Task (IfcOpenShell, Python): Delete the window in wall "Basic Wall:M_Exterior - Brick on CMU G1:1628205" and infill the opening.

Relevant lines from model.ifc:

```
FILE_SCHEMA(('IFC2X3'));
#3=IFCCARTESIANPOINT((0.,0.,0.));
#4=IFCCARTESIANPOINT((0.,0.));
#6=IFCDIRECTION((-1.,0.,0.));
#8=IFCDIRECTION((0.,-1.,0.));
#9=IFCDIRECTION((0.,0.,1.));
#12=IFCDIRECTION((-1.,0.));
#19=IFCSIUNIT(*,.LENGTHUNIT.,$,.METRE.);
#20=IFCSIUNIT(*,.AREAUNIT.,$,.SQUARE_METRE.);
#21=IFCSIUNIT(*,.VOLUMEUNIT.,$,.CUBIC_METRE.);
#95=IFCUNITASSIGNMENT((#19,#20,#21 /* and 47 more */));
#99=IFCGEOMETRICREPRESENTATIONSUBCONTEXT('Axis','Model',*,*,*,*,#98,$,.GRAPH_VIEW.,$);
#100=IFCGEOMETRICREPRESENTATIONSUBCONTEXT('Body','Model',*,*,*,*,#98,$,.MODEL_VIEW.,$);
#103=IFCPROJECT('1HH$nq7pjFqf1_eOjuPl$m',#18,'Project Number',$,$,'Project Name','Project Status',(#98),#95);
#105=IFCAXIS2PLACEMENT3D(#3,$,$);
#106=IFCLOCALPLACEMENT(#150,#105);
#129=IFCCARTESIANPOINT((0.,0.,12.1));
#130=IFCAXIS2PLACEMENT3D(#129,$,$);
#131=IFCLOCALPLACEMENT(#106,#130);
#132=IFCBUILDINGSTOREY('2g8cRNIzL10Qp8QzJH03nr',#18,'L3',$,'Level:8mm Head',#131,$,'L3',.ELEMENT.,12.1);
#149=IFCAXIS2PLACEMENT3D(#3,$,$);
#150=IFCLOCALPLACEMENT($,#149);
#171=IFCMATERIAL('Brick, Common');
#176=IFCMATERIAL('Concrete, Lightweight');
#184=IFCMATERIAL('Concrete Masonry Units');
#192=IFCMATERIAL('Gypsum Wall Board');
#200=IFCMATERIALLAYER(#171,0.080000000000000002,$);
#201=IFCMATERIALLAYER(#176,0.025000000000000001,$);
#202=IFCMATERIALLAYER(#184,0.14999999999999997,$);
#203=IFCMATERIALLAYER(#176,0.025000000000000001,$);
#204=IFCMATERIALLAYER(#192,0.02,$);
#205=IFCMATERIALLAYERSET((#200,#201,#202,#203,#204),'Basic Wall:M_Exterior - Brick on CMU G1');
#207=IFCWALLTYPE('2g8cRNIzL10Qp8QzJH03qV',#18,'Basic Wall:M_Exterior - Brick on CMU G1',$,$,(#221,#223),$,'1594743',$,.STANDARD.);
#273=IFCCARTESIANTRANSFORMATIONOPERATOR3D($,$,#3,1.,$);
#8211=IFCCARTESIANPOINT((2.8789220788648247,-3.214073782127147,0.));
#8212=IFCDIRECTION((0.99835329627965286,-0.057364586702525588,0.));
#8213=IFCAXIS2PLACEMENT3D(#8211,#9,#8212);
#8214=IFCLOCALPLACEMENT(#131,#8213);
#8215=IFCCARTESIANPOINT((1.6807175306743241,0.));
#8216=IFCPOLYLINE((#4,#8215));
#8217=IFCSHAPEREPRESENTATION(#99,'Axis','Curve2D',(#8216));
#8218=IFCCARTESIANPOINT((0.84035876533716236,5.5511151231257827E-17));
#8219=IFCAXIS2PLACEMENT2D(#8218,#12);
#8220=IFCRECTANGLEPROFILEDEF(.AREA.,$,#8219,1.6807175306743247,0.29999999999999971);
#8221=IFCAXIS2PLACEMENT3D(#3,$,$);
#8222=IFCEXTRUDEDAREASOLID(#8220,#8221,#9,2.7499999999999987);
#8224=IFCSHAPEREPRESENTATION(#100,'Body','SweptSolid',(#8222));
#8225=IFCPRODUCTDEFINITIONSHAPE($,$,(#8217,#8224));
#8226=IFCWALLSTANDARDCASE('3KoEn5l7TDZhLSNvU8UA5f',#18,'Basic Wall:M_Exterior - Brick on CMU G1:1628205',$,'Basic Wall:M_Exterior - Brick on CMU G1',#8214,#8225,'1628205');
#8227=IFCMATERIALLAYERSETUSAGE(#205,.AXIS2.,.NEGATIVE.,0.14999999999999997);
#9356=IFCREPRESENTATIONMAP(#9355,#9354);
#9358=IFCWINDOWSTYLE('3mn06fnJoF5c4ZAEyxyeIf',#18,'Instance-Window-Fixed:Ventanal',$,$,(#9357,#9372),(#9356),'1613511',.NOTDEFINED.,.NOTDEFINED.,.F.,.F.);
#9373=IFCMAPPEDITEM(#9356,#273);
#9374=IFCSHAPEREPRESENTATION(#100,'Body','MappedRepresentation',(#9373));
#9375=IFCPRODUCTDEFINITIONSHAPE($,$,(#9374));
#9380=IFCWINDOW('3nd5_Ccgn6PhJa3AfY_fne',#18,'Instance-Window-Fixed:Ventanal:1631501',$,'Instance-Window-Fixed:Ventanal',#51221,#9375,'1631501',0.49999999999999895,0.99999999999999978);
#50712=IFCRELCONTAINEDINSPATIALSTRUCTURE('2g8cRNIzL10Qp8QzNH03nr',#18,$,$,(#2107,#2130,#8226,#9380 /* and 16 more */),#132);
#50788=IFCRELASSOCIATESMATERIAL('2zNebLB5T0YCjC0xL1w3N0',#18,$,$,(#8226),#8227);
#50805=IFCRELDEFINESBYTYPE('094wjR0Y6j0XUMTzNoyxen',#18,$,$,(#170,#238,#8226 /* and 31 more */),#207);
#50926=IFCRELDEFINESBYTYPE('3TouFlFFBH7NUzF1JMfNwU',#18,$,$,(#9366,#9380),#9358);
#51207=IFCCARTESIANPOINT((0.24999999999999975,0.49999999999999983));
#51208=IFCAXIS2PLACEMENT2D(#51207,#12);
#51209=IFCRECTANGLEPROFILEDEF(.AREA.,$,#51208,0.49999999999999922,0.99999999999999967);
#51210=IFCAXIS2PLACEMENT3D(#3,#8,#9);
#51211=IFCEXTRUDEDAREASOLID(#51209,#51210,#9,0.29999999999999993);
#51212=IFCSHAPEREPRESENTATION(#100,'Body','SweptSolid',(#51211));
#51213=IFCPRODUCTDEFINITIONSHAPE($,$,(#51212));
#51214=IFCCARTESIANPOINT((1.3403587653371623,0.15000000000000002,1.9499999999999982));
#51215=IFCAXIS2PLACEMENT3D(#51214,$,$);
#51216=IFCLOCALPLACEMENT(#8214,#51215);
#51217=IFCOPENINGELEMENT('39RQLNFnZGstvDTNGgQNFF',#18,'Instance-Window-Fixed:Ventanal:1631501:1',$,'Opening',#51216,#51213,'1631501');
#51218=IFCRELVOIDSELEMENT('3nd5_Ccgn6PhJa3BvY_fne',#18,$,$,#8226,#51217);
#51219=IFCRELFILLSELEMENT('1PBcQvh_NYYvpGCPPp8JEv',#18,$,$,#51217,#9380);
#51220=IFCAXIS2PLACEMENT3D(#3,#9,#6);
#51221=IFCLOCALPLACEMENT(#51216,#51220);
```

```python
import ifcopenshell
import ifcopenshell.api.feature
import ifcopenshell.api.root
import ifcopenshell.geom
import ifcopenshell.util.shape

model = ifcopenshell.open("model.ifc")
settings = ifcopenshell.geom.settings()


def volume(element):
    """Net volume in cubic metres, openings subtracted."""
    shape = ifcopenshell.geom.create_shape(settings, element)
    return ifcopenshell.util.shape.get_volume(shape.geometry)


window = model.by_guid("3nd5_Ccgn6PhJa3AfY_fne")
opening = window.FillsVoids[0].RelatingOpeningElement
wall = opening.VoidsElements[0].RelatingBuildingElement
before = volume(wall)

ifcopenshell.api.root.remove_product(model, product=window)
ifcopenshell.api.feature.remove_feature(model, feature=opening)

after = volume(wall)

print(f"wall volume {before:.3f} -> {after:.3f} m3")

model.write("model_v2.ifc")
```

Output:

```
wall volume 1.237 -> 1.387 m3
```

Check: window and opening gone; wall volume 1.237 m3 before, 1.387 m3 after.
